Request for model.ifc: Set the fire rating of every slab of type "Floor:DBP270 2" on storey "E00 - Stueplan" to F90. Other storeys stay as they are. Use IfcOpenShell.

First a look at what the model holds.

```python
import ifcopenshell
import ifcopenshell.util.element

model = ifcopenshell.open("model.ifc")
print(model.schema)
storey = next(s for s in model.by_type("IfcBuildingStorey") if s.Name == "E00 - Stueplan")
slabs = [e for e in ifcopenshell.util.element.get_decomposition(storey) if e.is_a("IfcSlab")]
seen = {}
for e in slabs:
    element_type = ifcopenshell.util.element.get_type(e)
    key = (element_type.Name if element_type != e and element_type else None, ifcopenshell.util.element.get_pset(e, "Pset_SlabCommon", "FireRating"))
    seen[key] = seen.get(key, 0) + 1
for (name, value), count in sorted(seen.items(), key=str):
    print(count, "x", name, "|", value)
```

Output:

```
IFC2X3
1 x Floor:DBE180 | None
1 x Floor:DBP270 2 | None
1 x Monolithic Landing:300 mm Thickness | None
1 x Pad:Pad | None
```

```python
import ifcopenshell
import ifcopenshell.api.pset
import ifcopenshell.util.element

model = ifcopenshell.open("model.ifc")

storey = next(s for s in model.by_type("IfcBuildingStorey") if s.Name == "E00 - Stueplan")
slabs = [e for e in ifcopenshell.util.element.get_decomposition(storey) if e.is_a("IfcSlab")]

count = 0
for e in slabs:
    element_type = ifcopenshell.util.element.get_type(e)
    if element_type in (None, e) or element_type.Name != "Floor:DBP270 2":
        continue
    # add_pset returns the element's existing set when there is one.
    pset = ifcopenshell.api.pset.add_pset(model, product=e, name="Pset_SlabCommon")
    ifcopenshell.api.pset.edit_pset(model, pset=pset, properties={"FireRating": "F90"})
    count += 1

print(count, "slabs updated")

model.write("model_rev.ifc")
```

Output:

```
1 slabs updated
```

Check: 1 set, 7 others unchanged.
